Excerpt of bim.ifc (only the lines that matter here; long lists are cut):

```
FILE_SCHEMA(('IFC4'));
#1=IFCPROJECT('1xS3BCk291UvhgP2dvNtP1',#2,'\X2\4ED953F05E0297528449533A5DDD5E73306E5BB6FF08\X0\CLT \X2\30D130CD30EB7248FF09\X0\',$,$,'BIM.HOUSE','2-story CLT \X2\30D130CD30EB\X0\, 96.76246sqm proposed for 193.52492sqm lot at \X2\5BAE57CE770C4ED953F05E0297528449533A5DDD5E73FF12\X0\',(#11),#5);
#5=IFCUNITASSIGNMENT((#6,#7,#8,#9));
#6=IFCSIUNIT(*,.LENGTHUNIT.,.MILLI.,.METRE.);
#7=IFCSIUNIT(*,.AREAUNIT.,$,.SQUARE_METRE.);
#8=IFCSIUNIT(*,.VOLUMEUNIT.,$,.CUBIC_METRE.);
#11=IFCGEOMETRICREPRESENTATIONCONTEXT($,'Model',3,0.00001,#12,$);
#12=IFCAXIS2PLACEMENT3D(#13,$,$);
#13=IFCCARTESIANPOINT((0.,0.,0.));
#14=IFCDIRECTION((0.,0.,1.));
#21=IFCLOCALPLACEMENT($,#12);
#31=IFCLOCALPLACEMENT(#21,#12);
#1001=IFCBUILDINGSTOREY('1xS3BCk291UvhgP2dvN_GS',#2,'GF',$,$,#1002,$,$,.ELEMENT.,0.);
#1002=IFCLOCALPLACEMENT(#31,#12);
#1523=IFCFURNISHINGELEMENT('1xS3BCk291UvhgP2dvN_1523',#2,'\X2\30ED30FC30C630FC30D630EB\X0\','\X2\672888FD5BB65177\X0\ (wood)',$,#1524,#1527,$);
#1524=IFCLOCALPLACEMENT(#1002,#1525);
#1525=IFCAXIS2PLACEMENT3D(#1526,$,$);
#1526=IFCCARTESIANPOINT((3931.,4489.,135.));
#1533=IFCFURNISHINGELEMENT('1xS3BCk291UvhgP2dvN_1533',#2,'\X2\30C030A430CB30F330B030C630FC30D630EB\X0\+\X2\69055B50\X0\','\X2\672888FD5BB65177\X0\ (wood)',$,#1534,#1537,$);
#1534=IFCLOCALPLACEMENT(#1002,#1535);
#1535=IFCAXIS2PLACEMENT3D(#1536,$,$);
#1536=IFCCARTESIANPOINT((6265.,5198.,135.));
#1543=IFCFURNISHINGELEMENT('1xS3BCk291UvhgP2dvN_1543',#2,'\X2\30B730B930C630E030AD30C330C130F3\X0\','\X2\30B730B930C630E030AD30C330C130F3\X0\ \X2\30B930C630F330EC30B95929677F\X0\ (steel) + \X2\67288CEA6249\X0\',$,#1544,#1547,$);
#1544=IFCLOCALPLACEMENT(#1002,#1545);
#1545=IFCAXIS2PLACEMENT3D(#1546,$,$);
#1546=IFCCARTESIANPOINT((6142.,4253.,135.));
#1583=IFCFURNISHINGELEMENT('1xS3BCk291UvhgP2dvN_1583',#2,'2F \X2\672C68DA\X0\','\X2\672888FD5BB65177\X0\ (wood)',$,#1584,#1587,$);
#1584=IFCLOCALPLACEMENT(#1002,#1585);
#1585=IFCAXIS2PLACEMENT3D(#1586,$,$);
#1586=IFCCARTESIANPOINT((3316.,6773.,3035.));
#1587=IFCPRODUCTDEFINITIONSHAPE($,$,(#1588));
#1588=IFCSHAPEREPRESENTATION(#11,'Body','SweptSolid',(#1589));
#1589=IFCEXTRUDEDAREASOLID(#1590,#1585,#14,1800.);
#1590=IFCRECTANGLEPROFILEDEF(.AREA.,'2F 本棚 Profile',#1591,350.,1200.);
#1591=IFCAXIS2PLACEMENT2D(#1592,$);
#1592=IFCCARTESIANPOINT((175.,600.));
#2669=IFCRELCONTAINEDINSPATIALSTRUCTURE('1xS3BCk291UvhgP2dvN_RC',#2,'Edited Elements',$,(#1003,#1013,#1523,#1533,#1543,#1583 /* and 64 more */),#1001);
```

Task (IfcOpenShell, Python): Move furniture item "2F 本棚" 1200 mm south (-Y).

```python
import ifcopenshell
import ifcopenshell.api.geometry
import ifcopenshell.util.placement

model = ifcopenshell.open("bim.ifc")

item = model.by_id(1583)
matrix = ifcopenshell.util.placement.get_local_placement(item.ObjectPlacement)
matrix[1, 3] -= 1200.0
ifcopenshell.api.geometry.edit_object_placement(model, product=item, matrix=matrix, is_si=False)

print(ifcopenshell.util.placement.get_local_placement(item.ObjectPlacement).round(3) + 0.0)

model.write("bim_updated.ifc")
```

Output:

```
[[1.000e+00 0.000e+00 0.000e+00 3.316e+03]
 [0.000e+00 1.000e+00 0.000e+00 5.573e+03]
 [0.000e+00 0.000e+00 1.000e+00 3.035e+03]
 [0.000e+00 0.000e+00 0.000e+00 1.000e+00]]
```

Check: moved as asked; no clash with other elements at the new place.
